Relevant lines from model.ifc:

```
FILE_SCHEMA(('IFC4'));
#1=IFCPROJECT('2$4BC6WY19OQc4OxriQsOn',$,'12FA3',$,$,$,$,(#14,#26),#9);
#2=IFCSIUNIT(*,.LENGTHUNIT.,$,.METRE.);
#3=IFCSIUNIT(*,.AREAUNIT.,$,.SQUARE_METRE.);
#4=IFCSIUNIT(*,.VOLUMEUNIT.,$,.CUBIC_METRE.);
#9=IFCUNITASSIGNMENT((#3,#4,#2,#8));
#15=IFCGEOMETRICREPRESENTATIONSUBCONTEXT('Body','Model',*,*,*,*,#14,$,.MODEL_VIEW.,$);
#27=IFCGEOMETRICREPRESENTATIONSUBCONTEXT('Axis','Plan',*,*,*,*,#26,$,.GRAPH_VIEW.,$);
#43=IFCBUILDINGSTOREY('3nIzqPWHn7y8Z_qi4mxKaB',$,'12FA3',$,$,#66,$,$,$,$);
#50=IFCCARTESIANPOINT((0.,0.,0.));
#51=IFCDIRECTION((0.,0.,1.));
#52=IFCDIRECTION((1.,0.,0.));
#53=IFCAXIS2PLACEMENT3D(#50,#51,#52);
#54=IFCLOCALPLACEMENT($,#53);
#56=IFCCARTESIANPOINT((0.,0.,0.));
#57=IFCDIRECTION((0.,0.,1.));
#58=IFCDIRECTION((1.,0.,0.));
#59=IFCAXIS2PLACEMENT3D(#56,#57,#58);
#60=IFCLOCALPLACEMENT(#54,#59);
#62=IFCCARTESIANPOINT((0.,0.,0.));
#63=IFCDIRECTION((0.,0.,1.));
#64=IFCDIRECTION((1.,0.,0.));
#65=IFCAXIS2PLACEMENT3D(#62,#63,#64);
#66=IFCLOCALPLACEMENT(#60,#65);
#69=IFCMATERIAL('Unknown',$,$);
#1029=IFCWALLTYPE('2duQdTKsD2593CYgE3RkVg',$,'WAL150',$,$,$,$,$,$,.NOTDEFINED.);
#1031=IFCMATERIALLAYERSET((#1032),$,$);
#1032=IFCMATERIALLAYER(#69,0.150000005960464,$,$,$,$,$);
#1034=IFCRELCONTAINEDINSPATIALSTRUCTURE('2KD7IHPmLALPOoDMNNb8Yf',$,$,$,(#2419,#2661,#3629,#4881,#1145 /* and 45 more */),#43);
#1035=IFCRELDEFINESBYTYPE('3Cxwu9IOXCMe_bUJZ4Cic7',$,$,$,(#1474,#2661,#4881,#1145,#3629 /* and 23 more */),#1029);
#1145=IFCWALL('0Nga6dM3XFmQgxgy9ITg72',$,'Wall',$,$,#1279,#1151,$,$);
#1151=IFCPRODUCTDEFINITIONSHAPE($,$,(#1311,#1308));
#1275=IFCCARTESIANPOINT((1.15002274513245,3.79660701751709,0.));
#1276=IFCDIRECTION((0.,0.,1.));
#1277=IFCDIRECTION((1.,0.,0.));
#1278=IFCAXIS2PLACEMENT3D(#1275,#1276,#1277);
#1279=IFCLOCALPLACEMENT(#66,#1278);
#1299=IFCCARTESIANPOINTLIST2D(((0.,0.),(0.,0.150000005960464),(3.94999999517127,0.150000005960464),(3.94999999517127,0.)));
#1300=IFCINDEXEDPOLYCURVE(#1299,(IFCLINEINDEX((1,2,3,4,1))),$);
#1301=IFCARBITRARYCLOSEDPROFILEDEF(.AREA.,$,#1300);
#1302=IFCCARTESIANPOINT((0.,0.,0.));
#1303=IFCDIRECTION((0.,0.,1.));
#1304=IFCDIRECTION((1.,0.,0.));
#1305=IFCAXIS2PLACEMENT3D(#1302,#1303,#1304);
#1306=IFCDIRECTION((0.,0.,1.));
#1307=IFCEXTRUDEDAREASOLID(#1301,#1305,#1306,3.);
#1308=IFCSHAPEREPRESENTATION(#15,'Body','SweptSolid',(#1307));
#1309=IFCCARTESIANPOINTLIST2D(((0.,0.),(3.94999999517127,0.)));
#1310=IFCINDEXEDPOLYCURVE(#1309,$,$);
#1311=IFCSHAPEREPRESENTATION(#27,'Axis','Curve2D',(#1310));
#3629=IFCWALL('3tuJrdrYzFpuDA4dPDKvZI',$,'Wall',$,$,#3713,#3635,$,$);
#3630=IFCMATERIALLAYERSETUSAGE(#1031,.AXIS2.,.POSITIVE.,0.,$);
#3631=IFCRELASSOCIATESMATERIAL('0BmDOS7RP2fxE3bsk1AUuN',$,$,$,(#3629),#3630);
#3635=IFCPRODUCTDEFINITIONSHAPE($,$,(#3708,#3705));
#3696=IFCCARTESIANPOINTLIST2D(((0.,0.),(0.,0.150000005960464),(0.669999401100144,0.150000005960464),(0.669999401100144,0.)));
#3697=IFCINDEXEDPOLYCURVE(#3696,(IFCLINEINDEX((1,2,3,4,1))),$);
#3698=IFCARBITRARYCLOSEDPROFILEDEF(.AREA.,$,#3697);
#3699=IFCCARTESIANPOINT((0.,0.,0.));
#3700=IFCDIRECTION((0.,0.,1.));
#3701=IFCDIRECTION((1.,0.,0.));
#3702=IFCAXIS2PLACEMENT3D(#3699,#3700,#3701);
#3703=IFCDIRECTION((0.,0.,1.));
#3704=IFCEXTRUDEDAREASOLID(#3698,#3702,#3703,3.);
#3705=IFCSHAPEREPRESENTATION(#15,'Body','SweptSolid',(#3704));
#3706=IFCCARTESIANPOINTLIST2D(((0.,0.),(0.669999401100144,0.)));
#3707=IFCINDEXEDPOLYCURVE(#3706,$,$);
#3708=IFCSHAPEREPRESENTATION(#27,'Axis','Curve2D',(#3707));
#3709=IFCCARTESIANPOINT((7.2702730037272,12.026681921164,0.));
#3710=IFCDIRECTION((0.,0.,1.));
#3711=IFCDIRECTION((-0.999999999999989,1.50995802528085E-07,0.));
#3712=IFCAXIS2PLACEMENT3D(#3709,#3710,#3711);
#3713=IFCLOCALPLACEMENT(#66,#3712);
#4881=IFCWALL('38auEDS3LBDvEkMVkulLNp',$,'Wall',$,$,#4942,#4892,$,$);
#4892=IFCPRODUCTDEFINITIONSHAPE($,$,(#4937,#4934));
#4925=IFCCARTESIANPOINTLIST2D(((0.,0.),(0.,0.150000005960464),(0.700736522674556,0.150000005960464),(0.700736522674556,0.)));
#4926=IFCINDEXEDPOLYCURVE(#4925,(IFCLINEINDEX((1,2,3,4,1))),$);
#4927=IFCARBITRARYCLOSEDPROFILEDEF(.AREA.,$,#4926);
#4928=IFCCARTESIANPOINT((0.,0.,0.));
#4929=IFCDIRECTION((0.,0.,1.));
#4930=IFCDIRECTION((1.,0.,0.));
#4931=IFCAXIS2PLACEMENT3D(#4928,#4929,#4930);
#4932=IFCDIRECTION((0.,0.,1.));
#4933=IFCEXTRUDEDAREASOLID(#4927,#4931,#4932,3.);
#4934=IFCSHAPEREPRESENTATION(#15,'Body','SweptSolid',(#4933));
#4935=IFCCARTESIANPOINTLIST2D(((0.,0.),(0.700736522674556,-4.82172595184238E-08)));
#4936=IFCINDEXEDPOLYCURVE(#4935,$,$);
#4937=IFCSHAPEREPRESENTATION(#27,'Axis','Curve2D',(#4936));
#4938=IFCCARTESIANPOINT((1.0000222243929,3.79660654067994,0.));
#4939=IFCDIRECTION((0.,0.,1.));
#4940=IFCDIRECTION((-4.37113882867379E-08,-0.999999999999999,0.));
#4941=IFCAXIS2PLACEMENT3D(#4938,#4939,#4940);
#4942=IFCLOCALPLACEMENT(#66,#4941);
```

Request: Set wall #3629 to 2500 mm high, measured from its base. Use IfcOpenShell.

```python
import ifcopenshell
import ifcopenshell.geom
import ifcopenshell.util.representation
import ifcopenshell.util.shape

model = ifcopenshell.open("model.ifc")
settings = ifcopenshell.geom.settings()


def volume(element):
    """Net volume in cubic metres, openings subtracted."""
    shape = ifcopenshell.geom.create_shape(settings, element)
    return ifcopenshell.util.shape.get_volume(shape.geometry)


wall = model.by_id(3629)
before = volume(wall)

body = ifcopenshell.util.representation.get_representation(wall, "Model", "Body")
solid = body.Items[0]
old_height = solid.Depth
solid.Depth = 2.5
after = volume(wall)

print(f"height {old_height:g} -> {solid.Depth:g}, volume {before:.3f} -> {after:.3f} m3")

model.write("model_updated.ifc")
```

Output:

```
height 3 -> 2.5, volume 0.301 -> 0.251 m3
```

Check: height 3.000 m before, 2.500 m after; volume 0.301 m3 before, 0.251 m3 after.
